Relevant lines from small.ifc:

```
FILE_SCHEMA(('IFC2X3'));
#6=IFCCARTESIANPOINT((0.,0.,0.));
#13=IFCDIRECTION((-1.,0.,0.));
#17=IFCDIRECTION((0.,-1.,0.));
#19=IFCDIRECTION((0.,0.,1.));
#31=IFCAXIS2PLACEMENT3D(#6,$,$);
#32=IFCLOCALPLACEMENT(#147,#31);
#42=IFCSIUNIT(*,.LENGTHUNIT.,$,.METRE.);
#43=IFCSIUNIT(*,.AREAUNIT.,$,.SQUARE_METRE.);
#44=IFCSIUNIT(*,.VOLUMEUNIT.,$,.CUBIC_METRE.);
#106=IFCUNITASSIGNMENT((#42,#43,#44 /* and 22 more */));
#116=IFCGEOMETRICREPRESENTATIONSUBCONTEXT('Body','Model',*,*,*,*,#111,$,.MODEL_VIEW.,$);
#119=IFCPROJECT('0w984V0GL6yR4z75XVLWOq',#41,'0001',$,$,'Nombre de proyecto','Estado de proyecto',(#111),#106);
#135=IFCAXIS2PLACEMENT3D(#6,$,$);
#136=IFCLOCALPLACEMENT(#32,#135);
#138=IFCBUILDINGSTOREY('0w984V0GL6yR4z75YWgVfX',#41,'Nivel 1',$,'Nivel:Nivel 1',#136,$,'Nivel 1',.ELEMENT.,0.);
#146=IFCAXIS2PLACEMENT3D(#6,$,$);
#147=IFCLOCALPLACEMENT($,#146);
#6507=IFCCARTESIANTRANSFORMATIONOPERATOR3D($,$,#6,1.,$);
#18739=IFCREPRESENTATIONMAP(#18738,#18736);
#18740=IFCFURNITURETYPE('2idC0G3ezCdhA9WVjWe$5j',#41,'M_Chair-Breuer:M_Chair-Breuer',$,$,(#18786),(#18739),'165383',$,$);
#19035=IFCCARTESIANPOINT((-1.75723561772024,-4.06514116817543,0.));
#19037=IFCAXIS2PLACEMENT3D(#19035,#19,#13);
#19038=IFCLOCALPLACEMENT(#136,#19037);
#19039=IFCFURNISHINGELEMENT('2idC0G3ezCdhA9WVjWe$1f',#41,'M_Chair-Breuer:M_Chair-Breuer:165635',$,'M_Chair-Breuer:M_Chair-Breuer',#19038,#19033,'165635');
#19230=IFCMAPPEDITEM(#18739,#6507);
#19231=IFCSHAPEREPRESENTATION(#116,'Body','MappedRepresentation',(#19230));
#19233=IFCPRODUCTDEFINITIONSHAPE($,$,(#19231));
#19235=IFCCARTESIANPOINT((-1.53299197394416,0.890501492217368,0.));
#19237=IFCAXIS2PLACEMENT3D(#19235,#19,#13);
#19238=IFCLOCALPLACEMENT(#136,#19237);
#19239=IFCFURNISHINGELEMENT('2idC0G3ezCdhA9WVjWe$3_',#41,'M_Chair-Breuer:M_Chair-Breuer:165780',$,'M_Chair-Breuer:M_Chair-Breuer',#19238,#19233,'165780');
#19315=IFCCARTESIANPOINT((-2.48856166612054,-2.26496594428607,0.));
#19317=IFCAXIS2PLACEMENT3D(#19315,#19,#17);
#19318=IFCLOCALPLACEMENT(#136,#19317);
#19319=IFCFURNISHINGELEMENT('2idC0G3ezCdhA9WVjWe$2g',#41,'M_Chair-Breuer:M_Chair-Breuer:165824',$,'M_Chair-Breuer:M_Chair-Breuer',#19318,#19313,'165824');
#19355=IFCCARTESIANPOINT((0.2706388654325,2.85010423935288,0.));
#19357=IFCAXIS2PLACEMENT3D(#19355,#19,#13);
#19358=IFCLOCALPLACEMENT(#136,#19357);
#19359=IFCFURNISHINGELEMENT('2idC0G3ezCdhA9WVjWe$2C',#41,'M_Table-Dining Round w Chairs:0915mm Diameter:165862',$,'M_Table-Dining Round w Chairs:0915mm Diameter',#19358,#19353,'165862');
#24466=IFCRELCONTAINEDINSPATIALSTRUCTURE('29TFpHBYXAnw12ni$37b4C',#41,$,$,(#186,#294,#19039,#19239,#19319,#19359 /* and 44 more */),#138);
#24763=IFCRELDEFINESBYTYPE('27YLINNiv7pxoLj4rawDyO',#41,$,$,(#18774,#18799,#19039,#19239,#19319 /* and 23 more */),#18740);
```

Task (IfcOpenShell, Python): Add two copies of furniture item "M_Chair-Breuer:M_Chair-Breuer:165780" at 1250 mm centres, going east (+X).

```python
import numpy as np
import ifcopenshell
import ifcopenshell.api.geometry
import ifcopenshell.api.root
import ifcopenshell.util.element
import ifcopenshell.util.placement
import ifcopenshell.util.unit

model = ifcopenshell.open("small.ifc")
unit_scale = ifcopenshell.util.unit.calculate_unit_scale(model)


def reuse_history(source, copy):
    """copy_class also copies each property set's owner history, people and application; keep the originals."""
    for rel in copy.IsDefinedBy:
        if rel.is_a("IfcRelDefinesByProperties") and (history := rel.RelatingPropertyDefinition.OwnerHistory):
            rel.RelatingPropertyDefinition.OwnerHistory = source.OwnerHistory
            ifcopenshell.util.element.remove_deep2(model, history)


source = model.by_guid("2idC0G3ezCdhA9WVjWe$3_")
base = ifcopenshell.util.placement.get_local_placement(source.ObjectPlacement)
step = np.array([1.0, 0.0, 0.0]) * 1.25 / unit_scale

for i in range(1, 3):
    copy = ifcopenshell.api.root.copy_class(model, product=source)
    copy.Representation = ifcopenshell.util.element.copy_deep(
        model, source.Representation, exclude=["IfcGeometricRepresentationContext", "IfcRepresentationMap"]
    )
    copy.Name = "M_Chair-Breuer:M_Chair-Breuer"
    copy.Tag = None
    reuse_history(source, copy)
    matrix = base.copy()
    matrix[:3, 3] += i * step
    print("added at", matrix[:3, 3].round(3) + 0.0)
    ifcopenshell.api.geometry.edit_object_placement(model, product=copy, matrix=matrix, is_si=False)

model.write("small_updated.ifc")
```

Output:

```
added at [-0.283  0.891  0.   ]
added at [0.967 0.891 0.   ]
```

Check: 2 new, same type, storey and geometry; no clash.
